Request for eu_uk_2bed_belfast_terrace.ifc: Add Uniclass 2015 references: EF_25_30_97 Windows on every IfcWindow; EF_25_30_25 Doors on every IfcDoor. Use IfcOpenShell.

First a look at what the model holds.

```python
import ifcopenshell

model = ifcopenshell.open("eu_uk_2bed_belfast_terrace.ifc")
print(model.schema)
print("classifications:", [c.Name for c in model.by_type("IfcClassification")])
for ifc_class in ("IfcDoor", "IfcRoof", "IfcStair", "IfcWall", "IfcWindow"):
    print(ifc_class, len(model.by_type(ifc_class)))
```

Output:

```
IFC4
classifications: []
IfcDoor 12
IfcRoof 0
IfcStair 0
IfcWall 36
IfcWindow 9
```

```python
import ifcopenshell
import ifcopenshell.api.classification

model = ifcopenshell.open("eu_uk_2bed_belfast_terrace.ifc")

system = ifcopenshell.api.classification.add_classification(model, classification="Uniclass 2015")

codes = {
    "IfcWindow": ("EF_25_30_97", "Windows"),
    "IfcDoor": ("EF_25_30_25", "Doors"),
}
for ifc_class, (code, name) in codes.items():
    products = model.by_type(ifc_class)
    ifcopenshell.api.classification.add_reference(
        model, products=products, classification=system, identification=code, name=name
    )
    print(code, len(products))

model.write("eu_uk_2bed_belfast_terrace_v2.ifc")
```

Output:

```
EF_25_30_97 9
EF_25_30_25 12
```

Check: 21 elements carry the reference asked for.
